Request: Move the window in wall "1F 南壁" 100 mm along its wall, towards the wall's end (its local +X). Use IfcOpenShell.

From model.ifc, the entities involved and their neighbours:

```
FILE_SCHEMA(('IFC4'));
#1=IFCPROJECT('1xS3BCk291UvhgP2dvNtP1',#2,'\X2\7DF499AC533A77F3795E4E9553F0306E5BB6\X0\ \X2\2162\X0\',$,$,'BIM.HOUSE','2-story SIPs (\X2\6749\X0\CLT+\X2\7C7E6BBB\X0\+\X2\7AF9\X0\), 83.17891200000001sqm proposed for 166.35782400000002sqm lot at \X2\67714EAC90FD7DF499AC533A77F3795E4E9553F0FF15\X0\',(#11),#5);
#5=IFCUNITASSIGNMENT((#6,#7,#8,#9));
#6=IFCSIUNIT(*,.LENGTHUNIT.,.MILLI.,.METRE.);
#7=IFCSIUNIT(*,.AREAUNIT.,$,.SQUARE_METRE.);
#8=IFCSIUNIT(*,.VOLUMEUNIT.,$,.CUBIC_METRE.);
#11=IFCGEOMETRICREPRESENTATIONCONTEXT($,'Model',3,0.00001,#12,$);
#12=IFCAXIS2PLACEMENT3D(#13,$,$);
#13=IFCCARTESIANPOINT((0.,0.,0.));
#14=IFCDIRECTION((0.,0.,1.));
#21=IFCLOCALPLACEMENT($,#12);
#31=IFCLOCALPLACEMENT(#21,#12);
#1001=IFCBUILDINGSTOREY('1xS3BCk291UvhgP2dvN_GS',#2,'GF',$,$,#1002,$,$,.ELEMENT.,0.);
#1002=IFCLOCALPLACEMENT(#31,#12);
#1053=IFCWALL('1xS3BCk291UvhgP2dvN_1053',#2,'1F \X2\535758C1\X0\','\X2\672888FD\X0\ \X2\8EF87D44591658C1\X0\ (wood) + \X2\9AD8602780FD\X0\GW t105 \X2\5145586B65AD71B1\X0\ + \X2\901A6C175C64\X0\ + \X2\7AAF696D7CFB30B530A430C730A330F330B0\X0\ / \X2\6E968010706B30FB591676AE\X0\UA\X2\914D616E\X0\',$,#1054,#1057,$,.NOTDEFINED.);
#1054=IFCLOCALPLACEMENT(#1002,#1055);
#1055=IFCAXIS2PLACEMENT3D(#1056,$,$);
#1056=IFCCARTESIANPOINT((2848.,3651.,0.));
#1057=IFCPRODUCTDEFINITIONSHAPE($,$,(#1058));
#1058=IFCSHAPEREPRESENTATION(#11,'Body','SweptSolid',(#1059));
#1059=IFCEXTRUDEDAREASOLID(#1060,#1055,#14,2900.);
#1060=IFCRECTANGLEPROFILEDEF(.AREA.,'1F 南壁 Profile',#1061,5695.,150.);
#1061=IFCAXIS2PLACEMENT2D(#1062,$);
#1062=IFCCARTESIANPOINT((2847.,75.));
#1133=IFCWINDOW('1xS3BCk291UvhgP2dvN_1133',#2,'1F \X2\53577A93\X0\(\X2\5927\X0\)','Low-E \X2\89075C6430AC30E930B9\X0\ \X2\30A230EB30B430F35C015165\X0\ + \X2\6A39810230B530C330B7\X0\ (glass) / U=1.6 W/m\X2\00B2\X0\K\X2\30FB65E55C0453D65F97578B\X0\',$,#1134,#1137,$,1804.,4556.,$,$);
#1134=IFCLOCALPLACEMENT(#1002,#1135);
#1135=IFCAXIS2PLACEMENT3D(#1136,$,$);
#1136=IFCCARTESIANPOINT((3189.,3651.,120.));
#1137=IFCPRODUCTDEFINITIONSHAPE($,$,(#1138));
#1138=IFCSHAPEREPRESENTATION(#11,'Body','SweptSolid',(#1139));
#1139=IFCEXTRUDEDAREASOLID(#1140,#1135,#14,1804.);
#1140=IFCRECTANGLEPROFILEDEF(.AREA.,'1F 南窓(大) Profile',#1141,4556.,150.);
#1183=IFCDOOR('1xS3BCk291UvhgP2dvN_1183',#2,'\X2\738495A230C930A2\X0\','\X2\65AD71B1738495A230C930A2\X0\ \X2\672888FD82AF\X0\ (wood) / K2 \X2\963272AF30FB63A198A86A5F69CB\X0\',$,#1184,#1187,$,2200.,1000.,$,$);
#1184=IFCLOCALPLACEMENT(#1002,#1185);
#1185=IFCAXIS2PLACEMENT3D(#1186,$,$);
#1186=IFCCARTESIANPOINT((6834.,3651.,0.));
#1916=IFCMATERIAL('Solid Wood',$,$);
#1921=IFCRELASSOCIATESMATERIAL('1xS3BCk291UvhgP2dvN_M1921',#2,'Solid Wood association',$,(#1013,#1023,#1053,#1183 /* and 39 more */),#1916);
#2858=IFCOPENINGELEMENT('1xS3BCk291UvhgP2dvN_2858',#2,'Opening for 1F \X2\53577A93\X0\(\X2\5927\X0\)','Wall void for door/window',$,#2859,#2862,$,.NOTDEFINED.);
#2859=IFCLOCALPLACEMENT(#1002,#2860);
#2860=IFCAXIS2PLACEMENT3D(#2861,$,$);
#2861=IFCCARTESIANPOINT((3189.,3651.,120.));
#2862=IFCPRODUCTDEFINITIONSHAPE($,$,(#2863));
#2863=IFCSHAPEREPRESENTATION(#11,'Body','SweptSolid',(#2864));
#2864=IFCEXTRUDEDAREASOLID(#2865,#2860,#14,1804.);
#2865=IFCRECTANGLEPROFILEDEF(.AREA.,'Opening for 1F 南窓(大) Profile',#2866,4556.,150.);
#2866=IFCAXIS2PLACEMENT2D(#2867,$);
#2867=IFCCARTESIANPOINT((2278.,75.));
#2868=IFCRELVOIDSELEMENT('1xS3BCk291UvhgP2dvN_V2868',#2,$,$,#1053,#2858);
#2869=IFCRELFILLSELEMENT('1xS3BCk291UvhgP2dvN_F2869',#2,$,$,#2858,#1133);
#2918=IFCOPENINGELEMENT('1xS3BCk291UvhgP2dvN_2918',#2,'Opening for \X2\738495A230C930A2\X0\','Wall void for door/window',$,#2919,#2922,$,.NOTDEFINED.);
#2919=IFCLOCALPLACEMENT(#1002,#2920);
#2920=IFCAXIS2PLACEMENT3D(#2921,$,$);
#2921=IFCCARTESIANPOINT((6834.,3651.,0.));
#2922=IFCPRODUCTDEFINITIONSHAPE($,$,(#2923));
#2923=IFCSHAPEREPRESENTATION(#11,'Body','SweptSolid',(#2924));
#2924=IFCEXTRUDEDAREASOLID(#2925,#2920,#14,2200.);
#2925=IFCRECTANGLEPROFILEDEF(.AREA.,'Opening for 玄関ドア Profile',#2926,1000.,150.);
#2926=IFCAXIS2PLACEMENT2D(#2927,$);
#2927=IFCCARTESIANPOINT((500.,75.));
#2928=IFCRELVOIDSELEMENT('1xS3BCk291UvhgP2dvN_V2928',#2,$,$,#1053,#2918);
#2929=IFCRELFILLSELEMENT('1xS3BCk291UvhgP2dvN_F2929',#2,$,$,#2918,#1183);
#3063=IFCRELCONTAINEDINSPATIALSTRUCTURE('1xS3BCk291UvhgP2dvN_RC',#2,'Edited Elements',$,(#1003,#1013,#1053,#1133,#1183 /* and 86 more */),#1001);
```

```python
import ifcopenshell
import ifcopenshell.api.geometry
import ifcopenshell.util.placement
import ifcopenshell.util.unit

model = ifcopenshell.open("model.ifc")
unit_scale = ifcopenshell.util.unit.calculate_unit_scale(model)

window = model.by_guid("1xS3BCk291UvhgP2dvN_1133")
opening = window.FillsVoids[0].RelatingOpeningElement
wall = opening.VoidsElements[0].RelatingBuildingElement

wall_matrix = ifcopenshell.util.placement.get_local_placement(wall.ObjectPlacement)
shift = wall_matrix[:3, 0] * 0.1 / unit_scale
before = ifcopenshell.util.placement.get_local_placement(window.ObjectPlacement)[:3, 3].copy()

# The window is not placed relative to its opening, so move both.
for product in (opening, window):
    matrix = ifcopenshell.util.placement.get_local_placement(product.ObjectPlacement)
    matrix[:3, 3] += shift
    ifcopenshell.api.geometry.edit_object_placement(model, product=product, matrix=matrix, is_si=False)

after = ifcopenshell.util.placement.get_local_placement(window.ObjectPlacement)[:3, 3]
print("window moved by", (after - before).round(3) + 0.0)

model.write("model_rev.ifc")
```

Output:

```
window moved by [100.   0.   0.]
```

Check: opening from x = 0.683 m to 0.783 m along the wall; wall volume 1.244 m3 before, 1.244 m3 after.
